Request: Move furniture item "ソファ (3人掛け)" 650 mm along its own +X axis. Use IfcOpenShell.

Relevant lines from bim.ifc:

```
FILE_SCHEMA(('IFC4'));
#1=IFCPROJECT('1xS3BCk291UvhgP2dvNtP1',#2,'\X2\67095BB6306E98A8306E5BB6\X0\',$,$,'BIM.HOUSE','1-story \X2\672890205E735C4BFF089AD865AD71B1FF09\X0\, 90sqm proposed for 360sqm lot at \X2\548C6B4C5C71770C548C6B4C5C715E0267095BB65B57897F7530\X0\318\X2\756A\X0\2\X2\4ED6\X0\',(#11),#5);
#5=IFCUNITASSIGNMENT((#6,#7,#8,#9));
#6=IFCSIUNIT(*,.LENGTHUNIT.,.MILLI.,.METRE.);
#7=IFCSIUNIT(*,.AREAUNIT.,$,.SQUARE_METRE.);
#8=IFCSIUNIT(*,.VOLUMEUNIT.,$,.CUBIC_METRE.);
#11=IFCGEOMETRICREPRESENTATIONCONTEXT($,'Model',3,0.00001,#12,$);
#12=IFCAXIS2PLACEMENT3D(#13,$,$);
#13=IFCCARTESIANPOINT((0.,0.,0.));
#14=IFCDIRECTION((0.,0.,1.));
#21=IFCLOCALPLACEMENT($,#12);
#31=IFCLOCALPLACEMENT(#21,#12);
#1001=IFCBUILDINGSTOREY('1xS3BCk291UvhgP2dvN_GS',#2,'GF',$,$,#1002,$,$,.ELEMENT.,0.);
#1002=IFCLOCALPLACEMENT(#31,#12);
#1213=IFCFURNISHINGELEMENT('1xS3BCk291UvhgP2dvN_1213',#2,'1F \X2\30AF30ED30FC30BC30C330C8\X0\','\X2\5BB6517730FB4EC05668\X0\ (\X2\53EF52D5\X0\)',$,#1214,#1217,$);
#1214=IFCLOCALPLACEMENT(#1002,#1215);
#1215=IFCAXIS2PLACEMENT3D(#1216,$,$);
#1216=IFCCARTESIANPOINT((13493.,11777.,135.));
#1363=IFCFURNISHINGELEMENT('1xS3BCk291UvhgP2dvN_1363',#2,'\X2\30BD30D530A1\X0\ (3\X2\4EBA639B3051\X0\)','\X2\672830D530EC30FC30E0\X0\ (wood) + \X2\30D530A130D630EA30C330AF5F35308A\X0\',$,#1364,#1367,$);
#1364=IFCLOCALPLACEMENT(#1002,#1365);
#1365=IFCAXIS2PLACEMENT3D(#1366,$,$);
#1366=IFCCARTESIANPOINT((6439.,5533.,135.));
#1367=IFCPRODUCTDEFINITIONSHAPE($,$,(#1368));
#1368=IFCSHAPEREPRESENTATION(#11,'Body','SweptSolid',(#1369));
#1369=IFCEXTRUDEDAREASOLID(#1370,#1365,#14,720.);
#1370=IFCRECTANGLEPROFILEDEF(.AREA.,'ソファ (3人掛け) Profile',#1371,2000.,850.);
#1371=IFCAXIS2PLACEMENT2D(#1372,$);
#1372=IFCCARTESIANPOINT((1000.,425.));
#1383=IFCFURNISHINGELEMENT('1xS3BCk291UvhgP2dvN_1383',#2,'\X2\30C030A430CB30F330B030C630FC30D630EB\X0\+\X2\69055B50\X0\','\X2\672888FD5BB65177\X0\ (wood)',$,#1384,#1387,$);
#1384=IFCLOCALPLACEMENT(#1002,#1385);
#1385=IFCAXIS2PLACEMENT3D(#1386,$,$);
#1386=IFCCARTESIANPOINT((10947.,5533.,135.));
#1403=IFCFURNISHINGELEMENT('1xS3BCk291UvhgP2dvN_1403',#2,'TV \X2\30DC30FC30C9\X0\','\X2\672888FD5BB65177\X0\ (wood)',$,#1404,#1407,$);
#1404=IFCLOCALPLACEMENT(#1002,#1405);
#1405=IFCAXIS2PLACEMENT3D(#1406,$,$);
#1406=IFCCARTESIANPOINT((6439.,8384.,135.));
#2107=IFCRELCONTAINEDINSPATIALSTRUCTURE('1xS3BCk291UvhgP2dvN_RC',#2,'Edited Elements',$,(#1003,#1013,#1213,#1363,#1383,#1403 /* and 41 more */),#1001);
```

```python
import ifcopenshell
import ifcopenshell.api.geometry
import ifcopenshell.util.placement
import ifcopenshell.util.unit

model = ifcopenshell.open("bim.ifc")
unit_scale = ifcopenshell.util.unit.calculate_unit_scale(model)

item = model.by_guid("1xS3BCk291UvhgP2dvN_1363")
matrix = ifcopenshell.util.placement.get_local_placement(item.ObjectPlacement)
matrix[:3, 3] += matrix[:3, 0] * 0.65 / unit_scale
ifcopenshell.api.geometry.edit_object_placement(model, product=item, matrix=matrix, is_si=False)

print(ifcopenshell.util.placement.get_local_placement(item.ObjectPlacement).round(3) + 0.0)

model.write("bim-out.ifc")
```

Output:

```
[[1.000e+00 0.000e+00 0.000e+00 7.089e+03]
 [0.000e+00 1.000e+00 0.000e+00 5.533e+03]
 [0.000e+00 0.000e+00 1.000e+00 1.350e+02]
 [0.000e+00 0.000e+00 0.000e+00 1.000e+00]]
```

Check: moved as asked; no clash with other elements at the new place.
